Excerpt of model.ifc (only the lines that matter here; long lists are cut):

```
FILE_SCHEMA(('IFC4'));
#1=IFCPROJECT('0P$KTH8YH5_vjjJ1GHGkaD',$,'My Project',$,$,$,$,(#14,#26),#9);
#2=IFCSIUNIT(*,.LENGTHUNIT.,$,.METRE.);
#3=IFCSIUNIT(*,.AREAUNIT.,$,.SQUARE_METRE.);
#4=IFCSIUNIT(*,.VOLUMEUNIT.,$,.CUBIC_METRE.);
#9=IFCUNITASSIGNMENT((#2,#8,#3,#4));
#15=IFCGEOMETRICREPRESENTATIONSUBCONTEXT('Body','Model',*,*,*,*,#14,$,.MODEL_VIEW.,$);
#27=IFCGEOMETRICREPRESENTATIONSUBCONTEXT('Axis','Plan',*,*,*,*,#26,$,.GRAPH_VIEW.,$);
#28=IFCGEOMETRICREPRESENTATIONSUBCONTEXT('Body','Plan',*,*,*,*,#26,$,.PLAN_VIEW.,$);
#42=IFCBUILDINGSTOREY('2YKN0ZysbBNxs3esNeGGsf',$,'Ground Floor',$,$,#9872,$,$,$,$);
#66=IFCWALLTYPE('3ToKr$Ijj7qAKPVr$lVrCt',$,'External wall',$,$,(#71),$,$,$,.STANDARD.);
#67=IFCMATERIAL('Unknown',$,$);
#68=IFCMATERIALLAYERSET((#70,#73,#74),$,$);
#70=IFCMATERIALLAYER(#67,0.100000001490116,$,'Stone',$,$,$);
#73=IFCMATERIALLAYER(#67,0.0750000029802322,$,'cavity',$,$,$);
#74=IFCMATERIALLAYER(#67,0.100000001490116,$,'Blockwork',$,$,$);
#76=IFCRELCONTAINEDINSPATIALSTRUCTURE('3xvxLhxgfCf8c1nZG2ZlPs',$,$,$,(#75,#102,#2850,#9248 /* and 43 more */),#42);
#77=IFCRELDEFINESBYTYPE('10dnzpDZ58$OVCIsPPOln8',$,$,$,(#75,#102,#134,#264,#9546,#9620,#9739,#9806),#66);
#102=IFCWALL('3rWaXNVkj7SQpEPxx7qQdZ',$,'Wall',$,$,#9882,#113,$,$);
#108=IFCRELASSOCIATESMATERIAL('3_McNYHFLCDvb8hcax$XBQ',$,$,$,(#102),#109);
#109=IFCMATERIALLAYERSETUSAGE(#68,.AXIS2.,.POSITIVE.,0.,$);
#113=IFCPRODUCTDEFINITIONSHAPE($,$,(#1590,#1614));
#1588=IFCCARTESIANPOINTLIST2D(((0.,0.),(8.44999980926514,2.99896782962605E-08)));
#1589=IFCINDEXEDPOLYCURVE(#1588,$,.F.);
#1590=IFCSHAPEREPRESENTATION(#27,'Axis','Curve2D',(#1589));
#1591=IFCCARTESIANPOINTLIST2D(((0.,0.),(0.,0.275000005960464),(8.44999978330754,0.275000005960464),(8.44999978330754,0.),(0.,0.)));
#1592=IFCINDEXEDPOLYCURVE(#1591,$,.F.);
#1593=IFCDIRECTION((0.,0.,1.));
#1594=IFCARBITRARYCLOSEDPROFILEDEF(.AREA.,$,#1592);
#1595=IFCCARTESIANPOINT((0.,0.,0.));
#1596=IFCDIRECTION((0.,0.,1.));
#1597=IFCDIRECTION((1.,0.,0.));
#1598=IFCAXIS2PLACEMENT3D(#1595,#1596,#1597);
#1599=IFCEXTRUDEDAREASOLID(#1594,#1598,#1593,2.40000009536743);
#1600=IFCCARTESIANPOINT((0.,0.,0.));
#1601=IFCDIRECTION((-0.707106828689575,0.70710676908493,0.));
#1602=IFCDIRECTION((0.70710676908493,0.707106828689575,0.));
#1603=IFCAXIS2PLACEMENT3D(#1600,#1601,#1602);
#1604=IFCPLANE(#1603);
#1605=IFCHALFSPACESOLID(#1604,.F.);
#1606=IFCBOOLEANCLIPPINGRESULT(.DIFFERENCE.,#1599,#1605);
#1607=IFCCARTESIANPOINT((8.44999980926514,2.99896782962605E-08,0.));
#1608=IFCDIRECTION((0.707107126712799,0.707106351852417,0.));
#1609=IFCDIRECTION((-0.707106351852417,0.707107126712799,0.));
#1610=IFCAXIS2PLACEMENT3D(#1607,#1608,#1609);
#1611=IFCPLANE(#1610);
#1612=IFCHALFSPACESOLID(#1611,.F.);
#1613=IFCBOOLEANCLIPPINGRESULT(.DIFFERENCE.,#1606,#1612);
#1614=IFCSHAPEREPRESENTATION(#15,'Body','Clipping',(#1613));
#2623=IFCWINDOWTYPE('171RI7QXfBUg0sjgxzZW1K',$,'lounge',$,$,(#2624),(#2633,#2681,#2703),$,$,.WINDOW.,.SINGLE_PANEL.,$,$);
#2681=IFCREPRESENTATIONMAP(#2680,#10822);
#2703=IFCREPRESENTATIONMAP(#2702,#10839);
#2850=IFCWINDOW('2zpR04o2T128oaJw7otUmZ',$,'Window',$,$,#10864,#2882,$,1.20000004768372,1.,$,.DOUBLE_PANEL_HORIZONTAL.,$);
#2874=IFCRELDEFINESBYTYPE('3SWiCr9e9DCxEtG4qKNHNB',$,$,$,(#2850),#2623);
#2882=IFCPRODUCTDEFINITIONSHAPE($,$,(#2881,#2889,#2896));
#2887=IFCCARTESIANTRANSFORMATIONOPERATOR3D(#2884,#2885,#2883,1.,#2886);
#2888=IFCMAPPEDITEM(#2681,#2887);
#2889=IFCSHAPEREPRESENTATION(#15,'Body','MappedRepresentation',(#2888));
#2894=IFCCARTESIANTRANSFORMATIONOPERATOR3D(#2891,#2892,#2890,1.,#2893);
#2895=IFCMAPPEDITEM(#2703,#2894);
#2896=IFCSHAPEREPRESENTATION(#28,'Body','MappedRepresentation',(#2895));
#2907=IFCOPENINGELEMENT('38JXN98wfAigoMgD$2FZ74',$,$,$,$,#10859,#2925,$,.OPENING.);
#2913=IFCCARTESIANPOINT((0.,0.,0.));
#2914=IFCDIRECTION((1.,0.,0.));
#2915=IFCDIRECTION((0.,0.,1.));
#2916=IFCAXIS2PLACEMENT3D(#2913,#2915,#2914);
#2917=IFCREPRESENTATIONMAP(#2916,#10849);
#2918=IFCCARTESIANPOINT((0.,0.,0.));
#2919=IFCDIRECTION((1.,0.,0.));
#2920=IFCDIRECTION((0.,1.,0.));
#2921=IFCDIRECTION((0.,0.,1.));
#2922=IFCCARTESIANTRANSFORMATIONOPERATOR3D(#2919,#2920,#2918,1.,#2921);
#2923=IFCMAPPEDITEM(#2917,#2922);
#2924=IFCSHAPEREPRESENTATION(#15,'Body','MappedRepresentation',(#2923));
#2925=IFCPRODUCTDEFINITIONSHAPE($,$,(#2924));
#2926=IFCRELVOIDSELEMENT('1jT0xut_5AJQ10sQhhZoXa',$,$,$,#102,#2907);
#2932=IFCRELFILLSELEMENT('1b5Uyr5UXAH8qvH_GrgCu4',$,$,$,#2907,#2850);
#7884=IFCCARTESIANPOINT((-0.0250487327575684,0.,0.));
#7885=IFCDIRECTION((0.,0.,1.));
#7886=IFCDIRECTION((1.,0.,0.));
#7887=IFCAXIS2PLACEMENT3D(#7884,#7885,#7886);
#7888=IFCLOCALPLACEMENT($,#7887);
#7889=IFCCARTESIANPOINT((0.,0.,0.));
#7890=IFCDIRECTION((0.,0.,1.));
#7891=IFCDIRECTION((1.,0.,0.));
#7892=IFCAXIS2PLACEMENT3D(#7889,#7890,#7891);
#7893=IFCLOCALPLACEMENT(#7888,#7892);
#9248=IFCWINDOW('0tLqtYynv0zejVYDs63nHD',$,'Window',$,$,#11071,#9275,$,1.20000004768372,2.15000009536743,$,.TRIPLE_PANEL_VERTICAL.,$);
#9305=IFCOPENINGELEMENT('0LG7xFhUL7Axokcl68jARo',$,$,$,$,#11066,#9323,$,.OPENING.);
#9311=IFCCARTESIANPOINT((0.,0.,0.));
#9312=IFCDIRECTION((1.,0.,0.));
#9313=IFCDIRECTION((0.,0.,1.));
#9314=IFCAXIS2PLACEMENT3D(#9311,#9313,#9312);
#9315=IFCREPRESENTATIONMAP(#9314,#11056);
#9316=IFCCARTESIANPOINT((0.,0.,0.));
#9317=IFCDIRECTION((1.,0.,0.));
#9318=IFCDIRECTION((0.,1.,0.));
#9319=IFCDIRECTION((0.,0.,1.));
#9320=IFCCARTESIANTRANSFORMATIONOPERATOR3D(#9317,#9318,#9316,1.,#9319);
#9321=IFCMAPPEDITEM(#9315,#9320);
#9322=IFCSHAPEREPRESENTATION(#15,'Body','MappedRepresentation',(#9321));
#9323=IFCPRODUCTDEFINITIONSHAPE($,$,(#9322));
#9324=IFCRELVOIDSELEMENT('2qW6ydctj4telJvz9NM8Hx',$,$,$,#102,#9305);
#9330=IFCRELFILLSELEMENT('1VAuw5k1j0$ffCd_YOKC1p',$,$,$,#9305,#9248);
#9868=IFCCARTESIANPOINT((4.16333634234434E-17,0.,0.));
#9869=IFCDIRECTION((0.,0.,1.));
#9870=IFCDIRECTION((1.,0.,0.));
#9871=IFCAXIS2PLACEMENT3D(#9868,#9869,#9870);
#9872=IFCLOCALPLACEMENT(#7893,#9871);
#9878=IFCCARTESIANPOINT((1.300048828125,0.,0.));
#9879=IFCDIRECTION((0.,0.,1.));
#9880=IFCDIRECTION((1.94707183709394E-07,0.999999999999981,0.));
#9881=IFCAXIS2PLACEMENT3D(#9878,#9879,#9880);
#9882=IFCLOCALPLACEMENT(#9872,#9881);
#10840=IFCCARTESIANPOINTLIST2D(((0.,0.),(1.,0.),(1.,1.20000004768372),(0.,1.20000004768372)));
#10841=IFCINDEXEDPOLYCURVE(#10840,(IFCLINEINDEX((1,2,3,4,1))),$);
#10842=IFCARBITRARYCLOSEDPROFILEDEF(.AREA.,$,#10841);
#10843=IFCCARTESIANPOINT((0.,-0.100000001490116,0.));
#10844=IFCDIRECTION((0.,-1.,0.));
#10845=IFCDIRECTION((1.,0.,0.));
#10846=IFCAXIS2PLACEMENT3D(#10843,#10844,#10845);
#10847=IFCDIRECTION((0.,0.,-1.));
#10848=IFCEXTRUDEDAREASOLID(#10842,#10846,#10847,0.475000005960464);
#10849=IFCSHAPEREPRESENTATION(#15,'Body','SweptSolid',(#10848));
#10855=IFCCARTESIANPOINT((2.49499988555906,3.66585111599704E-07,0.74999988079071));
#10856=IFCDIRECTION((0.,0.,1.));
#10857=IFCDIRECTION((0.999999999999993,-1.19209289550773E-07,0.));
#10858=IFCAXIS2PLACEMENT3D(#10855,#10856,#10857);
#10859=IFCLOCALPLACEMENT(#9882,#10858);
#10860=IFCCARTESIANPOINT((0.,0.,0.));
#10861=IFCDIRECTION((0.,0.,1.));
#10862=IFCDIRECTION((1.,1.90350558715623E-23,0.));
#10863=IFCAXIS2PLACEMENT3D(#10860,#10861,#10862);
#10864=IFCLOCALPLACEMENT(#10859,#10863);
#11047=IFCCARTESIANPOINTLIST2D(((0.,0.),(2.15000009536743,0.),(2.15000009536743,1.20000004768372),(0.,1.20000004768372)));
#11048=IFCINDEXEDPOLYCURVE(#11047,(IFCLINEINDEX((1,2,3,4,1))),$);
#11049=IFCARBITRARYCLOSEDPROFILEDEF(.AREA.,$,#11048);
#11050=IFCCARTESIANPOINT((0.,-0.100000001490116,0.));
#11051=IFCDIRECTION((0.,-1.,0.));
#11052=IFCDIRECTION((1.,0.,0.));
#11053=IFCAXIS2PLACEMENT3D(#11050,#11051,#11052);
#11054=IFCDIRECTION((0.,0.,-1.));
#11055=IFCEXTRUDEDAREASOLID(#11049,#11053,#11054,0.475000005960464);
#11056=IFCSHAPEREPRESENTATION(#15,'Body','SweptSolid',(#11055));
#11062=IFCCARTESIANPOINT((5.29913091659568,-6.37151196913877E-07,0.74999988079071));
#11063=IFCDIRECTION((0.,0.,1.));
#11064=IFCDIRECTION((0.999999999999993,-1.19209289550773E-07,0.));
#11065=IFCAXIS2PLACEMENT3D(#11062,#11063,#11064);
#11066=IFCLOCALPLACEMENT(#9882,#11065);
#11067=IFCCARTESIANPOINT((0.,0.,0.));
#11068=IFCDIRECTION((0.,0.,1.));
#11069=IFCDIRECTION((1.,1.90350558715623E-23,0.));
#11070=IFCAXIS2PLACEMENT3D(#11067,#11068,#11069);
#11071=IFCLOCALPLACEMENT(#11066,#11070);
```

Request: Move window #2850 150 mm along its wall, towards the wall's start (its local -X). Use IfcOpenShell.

```python
import ifcopenshell
import ifcopenshell.api.geometry
import ifcopenshell.util.placement

model = ifcopenshell.open("model.ifc")

window = model.by_guid("2zpR04o2T128oaJw7otUmZ")
opening = window.FillsVoids[0].RelatingOpeningElement
wall = opening.VoidsElements[0].RelatingBuildingElement

wall_matrix = ifcopenshell.util.placement.get_local_placement(wall.ObjectPlacement)
shift = wall_matrix[:3, 0] * -0.15
before = ifcopenshell.util.placement.get_local_placement(window.ObjectPlacement)[:3, 3].copy()

# The window is placed relative to its opening, so it follows when the opening moves.
matrix = ifcopenshell.util.placement.get_local_placement(opening.ObjectPlacement)
matrix[:3, 3] += shift
ifcopenshell.api.geometry.edit_object_placement(
    model, product=opening, matrix=matrix, is_si=False, should_transform_children=True
)

after = ifcopenshell.util.placement.get_local_placement(window.ObjectPlacement)[:3, 3]
print("window moved by", (after - before).round(3) + 0.0)

model.write("model_rev.ifc")
```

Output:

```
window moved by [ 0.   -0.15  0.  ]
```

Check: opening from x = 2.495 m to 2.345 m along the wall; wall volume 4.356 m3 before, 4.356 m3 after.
